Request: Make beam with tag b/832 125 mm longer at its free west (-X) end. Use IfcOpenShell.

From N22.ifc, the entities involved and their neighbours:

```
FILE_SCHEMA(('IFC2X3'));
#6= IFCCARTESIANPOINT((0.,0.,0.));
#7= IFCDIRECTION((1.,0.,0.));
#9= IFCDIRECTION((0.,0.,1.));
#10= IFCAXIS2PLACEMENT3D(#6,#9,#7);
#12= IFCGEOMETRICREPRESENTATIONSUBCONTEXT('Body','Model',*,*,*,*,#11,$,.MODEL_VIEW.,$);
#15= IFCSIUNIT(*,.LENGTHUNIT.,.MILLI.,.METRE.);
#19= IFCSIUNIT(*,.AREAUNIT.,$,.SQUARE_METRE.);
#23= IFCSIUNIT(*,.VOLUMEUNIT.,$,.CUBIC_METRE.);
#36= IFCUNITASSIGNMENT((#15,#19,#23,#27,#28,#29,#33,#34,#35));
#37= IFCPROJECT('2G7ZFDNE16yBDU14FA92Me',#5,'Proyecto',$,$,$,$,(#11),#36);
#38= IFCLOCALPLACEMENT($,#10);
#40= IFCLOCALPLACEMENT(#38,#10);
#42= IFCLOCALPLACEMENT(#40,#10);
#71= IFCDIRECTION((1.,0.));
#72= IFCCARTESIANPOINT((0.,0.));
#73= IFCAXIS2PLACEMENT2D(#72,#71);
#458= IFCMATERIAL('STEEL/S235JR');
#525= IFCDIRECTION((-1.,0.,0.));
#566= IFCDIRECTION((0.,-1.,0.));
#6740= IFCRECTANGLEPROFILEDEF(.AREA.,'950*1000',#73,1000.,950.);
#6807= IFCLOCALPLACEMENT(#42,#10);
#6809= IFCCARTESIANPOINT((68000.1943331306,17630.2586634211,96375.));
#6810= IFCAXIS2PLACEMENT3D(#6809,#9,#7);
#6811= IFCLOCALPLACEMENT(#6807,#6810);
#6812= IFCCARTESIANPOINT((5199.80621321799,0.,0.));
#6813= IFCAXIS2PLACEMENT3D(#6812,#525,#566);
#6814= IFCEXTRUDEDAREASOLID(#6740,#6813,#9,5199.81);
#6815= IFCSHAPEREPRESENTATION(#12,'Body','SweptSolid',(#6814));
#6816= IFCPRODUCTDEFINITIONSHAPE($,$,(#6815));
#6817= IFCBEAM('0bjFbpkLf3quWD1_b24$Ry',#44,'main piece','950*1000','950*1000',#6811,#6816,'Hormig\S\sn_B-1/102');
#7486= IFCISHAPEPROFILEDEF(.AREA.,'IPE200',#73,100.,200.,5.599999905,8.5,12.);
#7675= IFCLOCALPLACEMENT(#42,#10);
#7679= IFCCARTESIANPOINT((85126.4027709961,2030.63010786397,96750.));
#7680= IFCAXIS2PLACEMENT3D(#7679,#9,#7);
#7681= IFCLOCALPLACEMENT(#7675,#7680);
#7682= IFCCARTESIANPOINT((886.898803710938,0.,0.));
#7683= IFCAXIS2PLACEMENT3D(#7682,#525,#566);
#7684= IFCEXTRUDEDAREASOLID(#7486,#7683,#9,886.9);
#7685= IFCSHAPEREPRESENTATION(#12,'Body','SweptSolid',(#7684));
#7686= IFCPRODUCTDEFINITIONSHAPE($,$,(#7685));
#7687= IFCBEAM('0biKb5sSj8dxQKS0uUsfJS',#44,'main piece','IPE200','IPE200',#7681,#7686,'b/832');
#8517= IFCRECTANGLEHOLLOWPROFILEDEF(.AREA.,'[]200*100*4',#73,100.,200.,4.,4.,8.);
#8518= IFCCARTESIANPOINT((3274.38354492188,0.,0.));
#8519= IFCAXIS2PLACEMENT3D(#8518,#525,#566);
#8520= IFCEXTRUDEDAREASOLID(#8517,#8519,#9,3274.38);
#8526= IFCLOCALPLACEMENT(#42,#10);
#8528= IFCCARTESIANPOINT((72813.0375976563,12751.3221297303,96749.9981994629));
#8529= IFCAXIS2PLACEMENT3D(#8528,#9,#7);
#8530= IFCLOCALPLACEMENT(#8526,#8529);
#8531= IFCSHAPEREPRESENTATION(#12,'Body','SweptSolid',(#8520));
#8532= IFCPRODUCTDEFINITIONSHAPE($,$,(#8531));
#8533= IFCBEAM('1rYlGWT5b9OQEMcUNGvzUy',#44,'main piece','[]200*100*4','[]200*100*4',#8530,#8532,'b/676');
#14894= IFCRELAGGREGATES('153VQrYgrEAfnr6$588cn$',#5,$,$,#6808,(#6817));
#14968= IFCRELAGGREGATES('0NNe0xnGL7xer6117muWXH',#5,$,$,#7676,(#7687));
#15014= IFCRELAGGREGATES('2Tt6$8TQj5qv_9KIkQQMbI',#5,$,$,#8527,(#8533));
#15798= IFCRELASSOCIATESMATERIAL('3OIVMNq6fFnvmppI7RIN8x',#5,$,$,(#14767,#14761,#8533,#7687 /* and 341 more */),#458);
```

```python
import ifcopenshell
import ifcopenshell.util.representation

model = ifcopenshell.open("N22.ifc")

member = model.by_guid("0biKb5sSj8dxQKS0uUsfJS")
change = 125.0

# The extrusion runs towards the end named, so only its depth changes.
body = ifcopenshell.util.representation.get_representation(member, "Model", "Body")
solid = body.Items[0]
old_length = solid.Depth
solid.Depth += change

print(f"length {old_length:g} -> {solid.Depth:g}")

model.write("N22_edited.ifc")
```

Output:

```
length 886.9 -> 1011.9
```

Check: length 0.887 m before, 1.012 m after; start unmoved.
